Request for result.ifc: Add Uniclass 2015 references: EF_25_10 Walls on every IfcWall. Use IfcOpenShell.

First a look at what the model holds.

```python
import ifcopenshell

model = ifcopenshell.open("result.ifc")
print(model.schema)
print("classifications:", [c.Name for c in model.by_type("IfcClassification")])
for ifc_class in ("IfcDoor", "IfcRoof", "IfcStair", "IfcWall", "IfcWindow"):
    print(ifc_class, len(model.by_type(ifc_class)))
```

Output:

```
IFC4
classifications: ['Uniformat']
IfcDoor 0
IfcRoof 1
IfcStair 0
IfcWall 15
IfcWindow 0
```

```python
import ifcopenshell
import ifcopenshell.api.classification

model = ifcopenshell.open("result.ifc")

system = ifcopenshell.api.classification.add_classification(model, classification="Uniclass 2015")

codes = {
    "IfcWall": ("EF_25_10", "Walls"),
}
for ifc_class, (code, name) in codes.items():
    products = model.by_type(ifc_class)
    ifcopenshell.api.classification.add_reference(
        model, products=products, classification=system, identification=code, name=name
    )
    print(code, len(products))

model.write("result_updated.ifc")
```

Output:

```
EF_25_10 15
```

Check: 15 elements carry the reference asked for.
